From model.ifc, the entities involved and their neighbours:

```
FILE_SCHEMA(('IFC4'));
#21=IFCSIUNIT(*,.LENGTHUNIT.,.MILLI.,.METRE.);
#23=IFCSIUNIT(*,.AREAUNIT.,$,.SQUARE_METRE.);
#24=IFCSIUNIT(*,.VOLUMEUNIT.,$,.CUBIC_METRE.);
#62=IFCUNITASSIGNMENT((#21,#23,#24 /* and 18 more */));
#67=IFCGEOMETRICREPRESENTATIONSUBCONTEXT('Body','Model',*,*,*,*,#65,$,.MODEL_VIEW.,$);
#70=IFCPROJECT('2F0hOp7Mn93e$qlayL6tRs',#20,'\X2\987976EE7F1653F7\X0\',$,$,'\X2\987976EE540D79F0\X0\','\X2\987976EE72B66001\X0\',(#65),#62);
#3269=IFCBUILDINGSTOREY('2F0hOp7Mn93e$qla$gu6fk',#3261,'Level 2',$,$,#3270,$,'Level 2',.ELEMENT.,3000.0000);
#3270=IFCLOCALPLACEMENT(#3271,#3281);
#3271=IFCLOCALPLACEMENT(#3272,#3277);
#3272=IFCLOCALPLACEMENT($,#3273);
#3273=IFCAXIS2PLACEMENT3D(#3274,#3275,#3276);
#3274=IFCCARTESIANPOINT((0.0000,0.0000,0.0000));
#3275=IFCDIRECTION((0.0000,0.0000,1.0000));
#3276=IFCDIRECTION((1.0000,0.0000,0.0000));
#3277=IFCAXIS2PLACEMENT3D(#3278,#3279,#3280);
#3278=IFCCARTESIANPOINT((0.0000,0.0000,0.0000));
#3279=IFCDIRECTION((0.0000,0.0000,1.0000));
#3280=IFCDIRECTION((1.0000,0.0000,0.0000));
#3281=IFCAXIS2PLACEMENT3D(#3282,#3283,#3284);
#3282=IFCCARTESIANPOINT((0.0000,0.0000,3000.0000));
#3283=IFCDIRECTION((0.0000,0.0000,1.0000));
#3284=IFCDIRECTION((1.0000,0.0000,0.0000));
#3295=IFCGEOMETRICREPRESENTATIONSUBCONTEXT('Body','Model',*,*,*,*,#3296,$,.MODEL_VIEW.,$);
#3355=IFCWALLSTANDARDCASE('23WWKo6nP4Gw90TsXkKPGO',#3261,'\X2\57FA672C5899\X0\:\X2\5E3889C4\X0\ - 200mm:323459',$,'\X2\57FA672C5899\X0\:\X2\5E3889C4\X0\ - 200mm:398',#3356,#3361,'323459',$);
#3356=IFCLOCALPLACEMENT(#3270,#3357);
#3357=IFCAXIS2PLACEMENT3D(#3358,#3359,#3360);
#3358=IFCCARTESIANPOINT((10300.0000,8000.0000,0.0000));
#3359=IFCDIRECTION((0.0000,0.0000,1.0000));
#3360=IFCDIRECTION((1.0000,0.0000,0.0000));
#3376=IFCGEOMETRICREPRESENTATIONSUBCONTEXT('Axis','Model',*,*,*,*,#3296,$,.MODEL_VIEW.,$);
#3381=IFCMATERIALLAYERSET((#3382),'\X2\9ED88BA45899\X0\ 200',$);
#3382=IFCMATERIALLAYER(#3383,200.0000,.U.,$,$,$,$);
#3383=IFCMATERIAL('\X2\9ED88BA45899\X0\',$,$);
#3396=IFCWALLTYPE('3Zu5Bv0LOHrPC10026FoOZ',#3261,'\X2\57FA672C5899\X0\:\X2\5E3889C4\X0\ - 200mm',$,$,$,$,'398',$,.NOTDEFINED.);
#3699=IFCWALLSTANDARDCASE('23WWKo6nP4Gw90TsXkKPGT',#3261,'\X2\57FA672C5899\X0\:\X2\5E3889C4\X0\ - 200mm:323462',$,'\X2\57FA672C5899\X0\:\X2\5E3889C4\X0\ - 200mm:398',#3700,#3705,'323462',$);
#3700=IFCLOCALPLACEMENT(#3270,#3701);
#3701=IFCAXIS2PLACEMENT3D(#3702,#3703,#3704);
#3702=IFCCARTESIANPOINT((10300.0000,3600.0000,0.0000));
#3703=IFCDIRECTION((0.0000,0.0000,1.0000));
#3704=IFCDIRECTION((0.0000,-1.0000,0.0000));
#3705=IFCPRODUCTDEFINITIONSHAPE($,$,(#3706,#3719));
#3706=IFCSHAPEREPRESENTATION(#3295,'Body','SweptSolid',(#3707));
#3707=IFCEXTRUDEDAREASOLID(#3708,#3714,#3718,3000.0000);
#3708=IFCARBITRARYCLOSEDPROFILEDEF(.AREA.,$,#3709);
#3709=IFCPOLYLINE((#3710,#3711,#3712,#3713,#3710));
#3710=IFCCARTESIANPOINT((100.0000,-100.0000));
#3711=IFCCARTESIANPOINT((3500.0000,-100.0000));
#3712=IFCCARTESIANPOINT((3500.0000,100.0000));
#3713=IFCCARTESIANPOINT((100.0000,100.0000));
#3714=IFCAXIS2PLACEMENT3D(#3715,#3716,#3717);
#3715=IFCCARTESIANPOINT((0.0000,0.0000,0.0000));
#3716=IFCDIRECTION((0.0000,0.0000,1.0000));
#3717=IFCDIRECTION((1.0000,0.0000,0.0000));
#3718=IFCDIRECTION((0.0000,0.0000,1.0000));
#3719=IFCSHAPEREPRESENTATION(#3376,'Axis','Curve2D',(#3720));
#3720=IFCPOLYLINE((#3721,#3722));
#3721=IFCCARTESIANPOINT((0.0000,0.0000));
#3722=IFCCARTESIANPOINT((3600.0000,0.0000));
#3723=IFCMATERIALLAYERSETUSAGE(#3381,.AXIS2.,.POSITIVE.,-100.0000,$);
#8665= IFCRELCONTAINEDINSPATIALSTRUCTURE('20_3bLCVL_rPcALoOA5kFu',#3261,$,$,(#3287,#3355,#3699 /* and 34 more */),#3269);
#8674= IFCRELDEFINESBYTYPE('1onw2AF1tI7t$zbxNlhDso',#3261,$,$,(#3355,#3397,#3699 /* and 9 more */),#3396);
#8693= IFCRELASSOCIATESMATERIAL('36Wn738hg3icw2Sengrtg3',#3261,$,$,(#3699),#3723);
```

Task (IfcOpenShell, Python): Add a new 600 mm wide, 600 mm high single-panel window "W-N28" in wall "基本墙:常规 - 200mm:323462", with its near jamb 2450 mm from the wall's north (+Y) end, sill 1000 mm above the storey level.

```python
import numpy as np
import ifcopenshell
import ifcopenshell.api.feature
import ifcopenshell.api.geometry
import ifcopenshell.api.root
import ifcopenshell.api.spatial
import ifcopenshell.geom
import ifcopenshell.util.element
import ifcopenshell.util.placement
import ifcopenshell.util.representation
import ifcopenshell.util.shape
import ifcopenshell.util.unit

model = ifcopenshell.open("model.ifc")
unit_scale = ifcopenshell.util.unit.calculate_unit_scale(model)
settings = ifcopenshell.geom.settings()


def volume(element):
    """Net volume in cubic metres, openings subtracted."""
    shape = ifcopenshell.geom.create_shape(settings, element)
    return ifcopenshell.util.shape.get_volume(shape.geometry)


wall = model.by_guid("23WWKo6nP4Gw90TsXkKPGT")
storey = ifcopenshell.util.element.get_container(wall, ifc_class="IfcBuildingStorey")
context = ifcopenshell.util.representation.get_context(model, "Model", "Body", "MODEL_VIEW")
before = volume(wall)

width, height, from_end, sill = 0.6, 0.6, 2.45, 1  # metres

# The wall runs along its own X axis, and the end named is its -X end.
wall_shape = ifcopenshell.geom.create_shape(settings, wall)
x, y, z = ifcopenshell.util.shape.get_vertices(wall_shape.geometry).T
start = x.min() + from_end
face, thickness = float(y.min()), float(y.max() - y.min())
wall_matrix = ifcopenshell.util.placement.get_local_placement(wall.ObjectPlacement)
level = ifcopenshell.util.placement.get_local_placement(storey.ObjectPlacement)[2, 3]


def in_wall(x, y):
    """Placement at x, y metres in the wall's axes, at sill height."""
    matrix = wall_matrix.copy()
    matrix[:, 3] = wall_matrix @ np.array([x / unit_scale, y / unit_scale, 0.0, 1.0])
    matrix[2, 3] = level + sill / unit_scale
    return matrix


# Opening: a box that overshoots both wall faces by 50 mm.
opening = ifcopenshell.api.root.create_entity(model, ifc_class="IfcOpeningElement", predefined_type="OPENING")
box = ifcopenshell.api.geometry.add_wall_representation(
    model, context=context, length=width, height=height, thickness=thickness + 0.1
)
ifcopenshell.api.geometry.assign_representation(model, product=opening, representation=box)
ifcopenshell.api.geometry.edit_object_placement(model, product=opening, matrix=in_wall(start, face - 0.05), is_si=False)
ifcopenshell.api.feature.add_feature(model, feature=opening, element=wall)

window = ifcopenshell.api.root.create_entity(model, ifc_class="IfcWindow", name="W-N28", predefined_type="WINDOW")
window.OverallWidth, window.OverallHeight = width / unit_scale, height / unit_scale
window.PartitioningType = "SINGLE_PANEL"
body = ifcopenshell.api.geometry.add_window_representation(
    model,
    context=context,
    overall_width=window.OverallWidth,
    overall_height=window.OverallHeight,
    partition_type="SINGLE_PANEL",
)
ifcopenshell.api.geometry.assign_representation(model, product=window, representation=body)
ifcopenshell.api.spatial.assign_container(model, products=[window], relating_structure=storey)
ifcopenshell.api.feature.add_filling(model, opening=opening, element=window)

# Centre the window in the wall's thickness.
ifcopenshell.api.geometry.edit_object_placement(model, product=window, matrix=in_wall(start, face), is_si=False)
window_shape = ifcopenshell.geom.create_shape(settings, window)
depth = ifcopenshell.util.shape.get_vertices(window_shape.geometry)[:, 1]
offset = face + thickness / 2 - (depth.min() + depth.max()) / 2
ifcopenshell.api.geometry.edit_object_placement(model, product=window, matrix=in_wall(start, offset), is_si=False)

after = volume(wall)

print(f"wall volume {before:.3f} -> {after:.3f} m3")

model.write("model-out.ifc")
```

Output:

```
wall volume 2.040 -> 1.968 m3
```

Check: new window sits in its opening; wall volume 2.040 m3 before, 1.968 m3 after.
